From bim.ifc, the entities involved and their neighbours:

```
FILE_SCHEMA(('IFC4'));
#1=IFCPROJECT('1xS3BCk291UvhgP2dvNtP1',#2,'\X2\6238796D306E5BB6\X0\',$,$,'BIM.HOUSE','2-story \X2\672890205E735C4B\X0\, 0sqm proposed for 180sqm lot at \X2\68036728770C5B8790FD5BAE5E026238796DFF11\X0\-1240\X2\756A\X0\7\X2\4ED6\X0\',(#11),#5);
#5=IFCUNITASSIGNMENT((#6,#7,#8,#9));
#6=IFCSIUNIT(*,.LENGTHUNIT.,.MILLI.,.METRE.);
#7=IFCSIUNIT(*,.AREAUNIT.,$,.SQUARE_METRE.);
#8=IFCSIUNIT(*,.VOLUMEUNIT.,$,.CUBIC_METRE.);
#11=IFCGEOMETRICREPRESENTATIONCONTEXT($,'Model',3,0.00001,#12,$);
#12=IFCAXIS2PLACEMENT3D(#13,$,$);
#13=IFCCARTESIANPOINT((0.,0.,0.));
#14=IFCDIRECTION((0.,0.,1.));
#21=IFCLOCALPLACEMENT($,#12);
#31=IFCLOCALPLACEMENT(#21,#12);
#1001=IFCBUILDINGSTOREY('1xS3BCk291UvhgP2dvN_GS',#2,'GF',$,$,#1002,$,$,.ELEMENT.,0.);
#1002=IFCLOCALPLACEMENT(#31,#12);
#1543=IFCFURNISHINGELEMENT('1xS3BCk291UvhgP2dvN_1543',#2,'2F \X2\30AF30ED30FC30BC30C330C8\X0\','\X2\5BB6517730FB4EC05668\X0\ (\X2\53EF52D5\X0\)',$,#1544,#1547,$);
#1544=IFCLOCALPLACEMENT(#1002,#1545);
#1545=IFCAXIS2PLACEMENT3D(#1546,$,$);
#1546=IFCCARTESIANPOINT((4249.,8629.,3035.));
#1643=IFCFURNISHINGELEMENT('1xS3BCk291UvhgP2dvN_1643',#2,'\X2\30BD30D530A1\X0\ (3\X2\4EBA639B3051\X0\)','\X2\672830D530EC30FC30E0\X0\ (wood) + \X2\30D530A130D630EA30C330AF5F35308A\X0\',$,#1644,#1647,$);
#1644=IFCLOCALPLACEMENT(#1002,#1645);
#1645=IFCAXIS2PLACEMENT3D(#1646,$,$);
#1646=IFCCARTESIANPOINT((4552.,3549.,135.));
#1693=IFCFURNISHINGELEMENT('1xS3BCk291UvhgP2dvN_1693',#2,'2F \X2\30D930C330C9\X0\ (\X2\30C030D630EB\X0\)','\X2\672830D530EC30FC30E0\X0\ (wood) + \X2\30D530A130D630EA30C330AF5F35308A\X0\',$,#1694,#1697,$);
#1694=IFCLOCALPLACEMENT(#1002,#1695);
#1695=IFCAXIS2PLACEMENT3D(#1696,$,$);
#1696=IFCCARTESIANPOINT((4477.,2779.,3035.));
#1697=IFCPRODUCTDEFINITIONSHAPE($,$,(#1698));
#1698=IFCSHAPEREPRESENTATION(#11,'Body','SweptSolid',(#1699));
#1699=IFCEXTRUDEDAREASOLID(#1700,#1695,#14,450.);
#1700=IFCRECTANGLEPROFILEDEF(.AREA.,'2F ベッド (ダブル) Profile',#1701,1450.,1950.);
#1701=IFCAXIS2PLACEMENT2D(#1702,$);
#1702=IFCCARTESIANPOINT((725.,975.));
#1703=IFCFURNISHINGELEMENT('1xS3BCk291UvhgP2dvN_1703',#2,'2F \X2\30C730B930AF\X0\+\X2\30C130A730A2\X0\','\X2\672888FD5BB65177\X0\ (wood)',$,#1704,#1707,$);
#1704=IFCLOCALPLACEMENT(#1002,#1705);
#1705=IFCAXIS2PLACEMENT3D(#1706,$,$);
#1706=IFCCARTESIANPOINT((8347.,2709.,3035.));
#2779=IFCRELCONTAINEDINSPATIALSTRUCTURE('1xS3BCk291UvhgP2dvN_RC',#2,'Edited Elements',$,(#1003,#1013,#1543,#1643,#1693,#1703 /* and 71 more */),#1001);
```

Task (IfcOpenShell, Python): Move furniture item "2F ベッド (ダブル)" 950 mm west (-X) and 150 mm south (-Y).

```python
import ifcopenshell
import ifcopenshell.api.geometry
import ifcopenshell.util.placement

model = ifcopenshell.open("bim.ifc")

item = model.by_guid("1xS3BCk291UvhgP2dvN_1693")
matrix = ifcopenshell.util.placement.get_local_placement(item.ObjectPlacement)
matrix[0, 3] -= 950.0
matrix[1, 3] -= 150.0
ifcopenshell.api.geometry.edit_object_placement(model, product=item, matrix=matrix, is_si=False)

print(ifcopenshell.util.placement.get_local_placement(item.ObjectPlacement).round(3) + 0.0)

model.write("bim_rev.ifc")
```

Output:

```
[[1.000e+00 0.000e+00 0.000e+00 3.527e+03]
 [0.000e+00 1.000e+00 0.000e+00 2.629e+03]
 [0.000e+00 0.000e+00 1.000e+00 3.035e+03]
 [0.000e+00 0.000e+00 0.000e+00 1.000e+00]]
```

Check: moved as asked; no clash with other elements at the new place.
